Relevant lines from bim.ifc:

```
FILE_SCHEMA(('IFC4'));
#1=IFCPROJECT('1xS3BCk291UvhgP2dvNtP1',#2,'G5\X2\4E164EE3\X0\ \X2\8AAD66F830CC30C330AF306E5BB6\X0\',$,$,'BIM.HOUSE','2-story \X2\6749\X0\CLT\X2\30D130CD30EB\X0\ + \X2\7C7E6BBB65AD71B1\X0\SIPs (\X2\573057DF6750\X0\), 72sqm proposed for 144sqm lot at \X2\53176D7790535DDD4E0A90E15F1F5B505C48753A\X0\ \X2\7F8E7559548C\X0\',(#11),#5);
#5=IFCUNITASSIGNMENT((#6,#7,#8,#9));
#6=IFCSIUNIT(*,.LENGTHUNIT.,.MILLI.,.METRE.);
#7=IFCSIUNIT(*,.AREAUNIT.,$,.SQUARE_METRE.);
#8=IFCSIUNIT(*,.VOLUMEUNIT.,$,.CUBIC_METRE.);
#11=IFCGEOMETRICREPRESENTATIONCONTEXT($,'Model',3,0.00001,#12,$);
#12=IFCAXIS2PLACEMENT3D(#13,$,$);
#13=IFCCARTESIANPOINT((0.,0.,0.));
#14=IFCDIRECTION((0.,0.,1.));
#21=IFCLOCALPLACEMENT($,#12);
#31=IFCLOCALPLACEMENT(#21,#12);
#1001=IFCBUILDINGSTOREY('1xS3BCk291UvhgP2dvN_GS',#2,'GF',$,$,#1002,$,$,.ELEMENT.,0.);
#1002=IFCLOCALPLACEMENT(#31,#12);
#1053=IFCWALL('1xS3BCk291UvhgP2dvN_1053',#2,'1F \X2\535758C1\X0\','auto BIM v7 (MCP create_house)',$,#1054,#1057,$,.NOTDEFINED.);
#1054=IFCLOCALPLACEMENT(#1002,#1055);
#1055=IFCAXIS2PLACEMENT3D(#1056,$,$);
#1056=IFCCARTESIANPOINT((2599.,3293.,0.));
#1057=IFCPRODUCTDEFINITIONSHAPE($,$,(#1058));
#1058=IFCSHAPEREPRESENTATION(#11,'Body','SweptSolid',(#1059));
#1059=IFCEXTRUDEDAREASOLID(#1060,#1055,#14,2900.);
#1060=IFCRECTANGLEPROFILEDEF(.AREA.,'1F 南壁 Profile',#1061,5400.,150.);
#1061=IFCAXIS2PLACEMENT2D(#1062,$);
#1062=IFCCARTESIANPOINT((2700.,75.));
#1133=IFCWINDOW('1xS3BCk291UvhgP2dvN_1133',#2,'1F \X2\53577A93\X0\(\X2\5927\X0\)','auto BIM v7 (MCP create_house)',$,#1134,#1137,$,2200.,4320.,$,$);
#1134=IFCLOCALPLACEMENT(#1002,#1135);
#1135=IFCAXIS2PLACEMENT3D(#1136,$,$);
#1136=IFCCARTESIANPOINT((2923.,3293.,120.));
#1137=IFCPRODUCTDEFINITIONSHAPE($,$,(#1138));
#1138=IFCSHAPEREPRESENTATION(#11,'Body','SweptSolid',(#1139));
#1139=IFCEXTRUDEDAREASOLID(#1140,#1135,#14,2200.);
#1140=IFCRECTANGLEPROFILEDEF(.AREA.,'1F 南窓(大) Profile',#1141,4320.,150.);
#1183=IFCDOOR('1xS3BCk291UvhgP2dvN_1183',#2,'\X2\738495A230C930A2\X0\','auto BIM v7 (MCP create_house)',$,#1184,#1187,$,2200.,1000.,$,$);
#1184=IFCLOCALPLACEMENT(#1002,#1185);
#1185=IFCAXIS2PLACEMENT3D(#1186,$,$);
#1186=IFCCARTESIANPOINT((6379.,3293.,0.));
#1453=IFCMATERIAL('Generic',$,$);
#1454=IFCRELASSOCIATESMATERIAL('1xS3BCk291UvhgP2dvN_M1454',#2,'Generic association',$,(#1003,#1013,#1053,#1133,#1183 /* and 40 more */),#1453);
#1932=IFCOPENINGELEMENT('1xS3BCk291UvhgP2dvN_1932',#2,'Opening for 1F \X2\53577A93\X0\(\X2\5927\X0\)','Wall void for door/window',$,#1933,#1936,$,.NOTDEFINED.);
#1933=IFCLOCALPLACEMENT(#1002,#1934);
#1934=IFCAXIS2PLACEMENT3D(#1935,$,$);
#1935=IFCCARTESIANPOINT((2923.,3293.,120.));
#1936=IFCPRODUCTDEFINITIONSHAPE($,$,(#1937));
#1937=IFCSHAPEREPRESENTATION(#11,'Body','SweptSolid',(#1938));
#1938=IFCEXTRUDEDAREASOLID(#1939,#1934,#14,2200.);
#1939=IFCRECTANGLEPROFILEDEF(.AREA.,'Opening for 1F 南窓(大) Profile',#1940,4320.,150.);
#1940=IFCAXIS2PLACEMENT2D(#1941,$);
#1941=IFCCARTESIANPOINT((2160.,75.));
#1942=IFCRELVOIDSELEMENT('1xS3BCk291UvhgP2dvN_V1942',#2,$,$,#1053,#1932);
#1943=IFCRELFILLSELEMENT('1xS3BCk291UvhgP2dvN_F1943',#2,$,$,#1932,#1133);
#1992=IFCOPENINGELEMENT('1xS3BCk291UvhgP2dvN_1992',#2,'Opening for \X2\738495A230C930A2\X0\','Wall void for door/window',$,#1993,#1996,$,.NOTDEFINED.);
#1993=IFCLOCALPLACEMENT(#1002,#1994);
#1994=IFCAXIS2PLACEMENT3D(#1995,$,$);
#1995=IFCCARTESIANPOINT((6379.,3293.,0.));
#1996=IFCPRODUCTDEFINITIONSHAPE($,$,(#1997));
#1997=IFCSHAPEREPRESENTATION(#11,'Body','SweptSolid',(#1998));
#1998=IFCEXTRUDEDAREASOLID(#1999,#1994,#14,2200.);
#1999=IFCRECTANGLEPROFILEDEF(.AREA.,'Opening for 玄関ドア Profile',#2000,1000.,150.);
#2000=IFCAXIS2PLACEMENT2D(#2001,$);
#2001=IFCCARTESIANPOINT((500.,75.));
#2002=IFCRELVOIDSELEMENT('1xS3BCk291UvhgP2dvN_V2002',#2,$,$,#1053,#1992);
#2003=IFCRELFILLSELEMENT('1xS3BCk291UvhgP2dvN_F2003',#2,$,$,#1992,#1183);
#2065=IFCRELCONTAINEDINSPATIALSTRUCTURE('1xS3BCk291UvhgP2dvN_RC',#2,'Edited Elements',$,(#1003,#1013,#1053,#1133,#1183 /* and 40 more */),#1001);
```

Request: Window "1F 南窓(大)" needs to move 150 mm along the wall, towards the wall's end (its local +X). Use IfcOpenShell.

```python
import ifcopenshell
import ifcopenshell.api.geometry
import ifcopenshell.util.placement

model = ifcopenshell.open("bim.ifc")

window = model.by_guid("1xS3BCk291UvhgP2dvN_1133")
opening = window.FillsVoids[0].RelatingOpeningElement
wall = opening.VoidsElements[0].RelatingBuildingElement

wall_matrix = ifcopenshell.util.placement.get_local_placement(wall.ObjectPlacement)
shift = wall_matrix[:3, 0] * 150.0
before = ifcopenshell.util.placement.get_local_placement(window.ObjectPlacement)[:3, 3].copy()

# The window is not placed relative to its opening, so move both.
for product in (opening, window):
    matrix = ifcopenshell.util.placement.get_local_placement(product.ObjectPlacement)
    matrix[:3, 3] += shift
    ifcopenshell.api.geometry.edit_object_placement(model, product=product, matrix=matrix, is_si=False)

after = ifcopenshell.util.placement.get_local_placement(window.ObjectPlacement)[:3, 3]
print("window moved by", (after - before).round(3) + 0.0)

model.write("bim_updated.ifc")
```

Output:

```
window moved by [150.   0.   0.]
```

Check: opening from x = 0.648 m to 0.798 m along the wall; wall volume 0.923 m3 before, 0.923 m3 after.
